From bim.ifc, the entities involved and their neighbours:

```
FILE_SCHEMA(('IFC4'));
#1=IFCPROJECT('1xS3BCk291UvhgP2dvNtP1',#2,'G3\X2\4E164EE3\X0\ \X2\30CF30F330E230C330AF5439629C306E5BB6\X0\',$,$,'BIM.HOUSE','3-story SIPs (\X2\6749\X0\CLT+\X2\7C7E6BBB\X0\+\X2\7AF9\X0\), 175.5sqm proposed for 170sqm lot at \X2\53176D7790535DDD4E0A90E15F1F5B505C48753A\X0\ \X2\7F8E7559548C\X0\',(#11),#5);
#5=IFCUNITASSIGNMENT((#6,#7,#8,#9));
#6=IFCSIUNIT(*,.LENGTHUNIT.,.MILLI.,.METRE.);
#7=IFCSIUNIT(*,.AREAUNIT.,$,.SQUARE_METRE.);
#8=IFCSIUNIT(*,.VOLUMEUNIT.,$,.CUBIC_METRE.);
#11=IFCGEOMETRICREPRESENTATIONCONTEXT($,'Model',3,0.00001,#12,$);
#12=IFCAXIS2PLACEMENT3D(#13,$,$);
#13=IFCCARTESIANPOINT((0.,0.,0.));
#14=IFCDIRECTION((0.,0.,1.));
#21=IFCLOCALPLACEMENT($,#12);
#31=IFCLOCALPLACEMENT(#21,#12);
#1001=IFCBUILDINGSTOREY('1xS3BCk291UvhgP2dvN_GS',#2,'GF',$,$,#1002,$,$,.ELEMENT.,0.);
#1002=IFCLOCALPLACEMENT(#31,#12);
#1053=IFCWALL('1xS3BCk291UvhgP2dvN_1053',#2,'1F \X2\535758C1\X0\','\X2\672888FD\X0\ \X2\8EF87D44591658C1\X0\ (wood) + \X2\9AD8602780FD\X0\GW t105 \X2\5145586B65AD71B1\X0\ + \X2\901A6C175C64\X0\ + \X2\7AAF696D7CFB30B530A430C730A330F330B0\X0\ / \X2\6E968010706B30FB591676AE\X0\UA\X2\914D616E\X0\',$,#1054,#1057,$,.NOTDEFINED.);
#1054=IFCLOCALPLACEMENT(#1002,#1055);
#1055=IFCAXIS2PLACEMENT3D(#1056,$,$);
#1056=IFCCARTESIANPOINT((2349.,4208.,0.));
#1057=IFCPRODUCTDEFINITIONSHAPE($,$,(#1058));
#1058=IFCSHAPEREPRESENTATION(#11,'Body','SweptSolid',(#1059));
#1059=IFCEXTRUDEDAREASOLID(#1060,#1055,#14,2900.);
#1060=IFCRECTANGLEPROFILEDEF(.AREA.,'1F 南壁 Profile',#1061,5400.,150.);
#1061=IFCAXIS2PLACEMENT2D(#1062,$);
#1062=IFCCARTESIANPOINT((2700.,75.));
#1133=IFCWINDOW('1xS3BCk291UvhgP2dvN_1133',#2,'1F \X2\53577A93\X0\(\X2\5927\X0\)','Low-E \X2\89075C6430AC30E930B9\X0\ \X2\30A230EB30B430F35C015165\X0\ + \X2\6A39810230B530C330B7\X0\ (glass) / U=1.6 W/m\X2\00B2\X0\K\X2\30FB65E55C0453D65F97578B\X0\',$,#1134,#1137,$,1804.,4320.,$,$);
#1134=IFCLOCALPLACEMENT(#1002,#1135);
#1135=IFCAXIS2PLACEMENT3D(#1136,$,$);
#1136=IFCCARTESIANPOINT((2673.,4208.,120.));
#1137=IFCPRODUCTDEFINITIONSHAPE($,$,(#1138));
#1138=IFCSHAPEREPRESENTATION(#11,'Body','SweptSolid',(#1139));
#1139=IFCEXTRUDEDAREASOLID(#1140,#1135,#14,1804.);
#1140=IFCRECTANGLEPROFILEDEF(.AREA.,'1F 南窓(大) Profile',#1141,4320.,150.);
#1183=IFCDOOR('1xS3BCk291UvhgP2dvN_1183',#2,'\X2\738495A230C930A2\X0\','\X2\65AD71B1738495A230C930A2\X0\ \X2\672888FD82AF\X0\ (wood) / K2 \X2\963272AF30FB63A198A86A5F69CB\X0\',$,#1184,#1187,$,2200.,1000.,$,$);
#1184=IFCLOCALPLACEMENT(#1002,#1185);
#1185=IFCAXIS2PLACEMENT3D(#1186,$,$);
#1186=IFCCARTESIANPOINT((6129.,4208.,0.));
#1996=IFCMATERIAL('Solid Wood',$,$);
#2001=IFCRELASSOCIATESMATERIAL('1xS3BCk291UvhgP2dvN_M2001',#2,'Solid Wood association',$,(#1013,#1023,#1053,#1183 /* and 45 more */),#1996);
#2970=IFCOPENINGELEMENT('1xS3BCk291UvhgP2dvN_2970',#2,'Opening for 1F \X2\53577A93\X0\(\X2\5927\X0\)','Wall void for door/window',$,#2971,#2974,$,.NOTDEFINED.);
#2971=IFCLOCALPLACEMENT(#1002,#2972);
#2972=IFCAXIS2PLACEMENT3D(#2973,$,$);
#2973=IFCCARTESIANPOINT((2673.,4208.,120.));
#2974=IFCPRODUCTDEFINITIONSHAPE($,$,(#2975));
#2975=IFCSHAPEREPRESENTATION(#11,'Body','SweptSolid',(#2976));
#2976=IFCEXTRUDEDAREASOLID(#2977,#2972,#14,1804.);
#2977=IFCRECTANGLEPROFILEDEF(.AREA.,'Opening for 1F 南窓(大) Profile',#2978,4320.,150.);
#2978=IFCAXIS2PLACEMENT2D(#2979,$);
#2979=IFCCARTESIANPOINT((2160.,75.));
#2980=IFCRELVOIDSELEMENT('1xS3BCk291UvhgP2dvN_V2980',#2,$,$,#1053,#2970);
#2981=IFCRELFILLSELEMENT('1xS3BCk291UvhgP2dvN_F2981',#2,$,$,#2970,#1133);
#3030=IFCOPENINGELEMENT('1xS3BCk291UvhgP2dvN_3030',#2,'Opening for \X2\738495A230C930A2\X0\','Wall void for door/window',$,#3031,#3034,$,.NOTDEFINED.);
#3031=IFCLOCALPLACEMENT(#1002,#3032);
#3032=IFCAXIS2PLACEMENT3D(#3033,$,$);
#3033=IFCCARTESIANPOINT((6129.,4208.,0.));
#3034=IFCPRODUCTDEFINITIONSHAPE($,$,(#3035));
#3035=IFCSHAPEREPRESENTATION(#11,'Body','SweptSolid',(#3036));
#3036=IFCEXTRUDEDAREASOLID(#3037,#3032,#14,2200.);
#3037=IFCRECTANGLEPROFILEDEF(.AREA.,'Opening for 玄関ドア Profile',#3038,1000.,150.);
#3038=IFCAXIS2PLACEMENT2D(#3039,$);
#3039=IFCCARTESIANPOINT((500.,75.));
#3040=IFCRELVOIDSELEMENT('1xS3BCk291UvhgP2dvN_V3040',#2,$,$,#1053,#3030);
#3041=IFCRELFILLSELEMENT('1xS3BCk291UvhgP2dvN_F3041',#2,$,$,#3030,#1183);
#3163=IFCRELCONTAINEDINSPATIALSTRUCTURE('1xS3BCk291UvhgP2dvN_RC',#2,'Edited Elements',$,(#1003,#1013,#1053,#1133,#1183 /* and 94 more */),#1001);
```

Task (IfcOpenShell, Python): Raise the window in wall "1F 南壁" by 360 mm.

```python
import numpy as np
import ifcopenshell
import ifcopenshell.api.geometry
import ifcopenshell.util.placement
import ifcopenshell.util.unit

model = ifcopenshell.open("bim.ifc")
unit_scale = ifcopenshell.util.unit.calculate_unit_scale(model)

window = model.by_guid("1xS3BCk291UvhgP2dvN_1133")
opening = window.FillsVoids[0].RelatingOpeningElement
dz = 0.36 / unit_scale

shift = np.array([0.0, 0.0, dz])
# The window is not placed relative to its opening, so move both.
for product in (opening, window):
    matrix = ifcopenshell.util.placement.get_local_placement(product.ObjectPlacement)
    matrix[:3, 3] += shift
    ifcopenshell.api.geometry.edit_object_placement(model, product=product, matrix=matrix, is_si=False)

print(f"moved by {dz * unit_scale:+.3f} m")

model.write("bim_updated.ifc")
```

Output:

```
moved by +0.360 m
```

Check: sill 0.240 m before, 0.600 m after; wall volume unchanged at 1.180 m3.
